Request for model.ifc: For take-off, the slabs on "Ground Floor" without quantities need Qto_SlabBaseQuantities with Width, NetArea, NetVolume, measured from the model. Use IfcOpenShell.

First a look at what the model holds.

```python
import ifcopenshell
import ifcopenshell.util.element
import ifcopenshell.util.unit

model = ifcopenshell.open("model.ifc")
print(model.schema)
for unit_type in ("LENGTHUNIT", "AREAUNIT", "VOLUMEUNIT"):
    print(unit_type, ifcopenshell.util.unit.calculate_unit_scale(model, unit_type))
storey = next(s for s in model.by_type("IfcBuildingStorey") if s.Name == "Ground Floor")
slabs = [e for e in ifcopenshell.util.element.get_decomposition(storey) if e.is_a("IfcSlab")]
for e in sorted(slabs, key=lambda e: e.id()):
    print(e.id(), e.is_a(), e.Name, list(ifcopenshell.util.element.get_psets(e, qtos_only=True)), sep=" | ")
```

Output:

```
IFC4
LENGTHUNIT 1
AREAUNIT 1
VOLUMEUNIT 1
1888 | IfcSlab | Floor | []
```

```python
import ifcopenshell
import ifcopenshell.api.pset
import ifcopenshell.geom
import ifcopenshell.util.element
import ifcopenshell.util.shape
import ifcopenshell.util.unit

model = ifcopenshell.open("model.ifc")
unit_scale = ifcopenshell.util.unit.calculate_unit_scale(model)
area_scale = ifcopenshell.util.unit.calculate_unit_scale(model, "AREAUNIT")
volume_scale = ifcopenshell.util.unit.calculate_unit_scale(model, "VOLUMEUNIT")
settings = ifcopenshell.geom.settings()

storey = next(s for s in model.by_type("IfcBuildingStorey") if s.Name == "Ground Floor")
slabs = [e for e in ifcopenshell.util.element.get_decomposition(storey) if e.is_a("IfcSlab")]

for e in sorted(slabs, key=lambda e: e.id()):
    if ifcopenshell.util.element.get_psets(e, qtos_only=True, should_inherit=False):
        continue
    # Geometry comes back in metres, in the element's own axes.
    shape = ifcopenshell.geom.create_shape(settings, e)
    values = {
        "Width": ifcopenshell.util.shape.get_z(shape.geometry) / unit_scale,
        "NetArea": ifcopenshell.util.shape.get_footprint_area(shape.geometry) / area_scale,
        "NetVolume": ifcopenshell.util.shape.get_volume(shape.geometry) / volume_scale,
    }
    qto = ifcopenshell.api.pset.add_qto(model, product=e, name="Qto_SlabBaseQuantities")
    ifcopenshell.api.pset.edit_qto(model, qto=qto, properties=values)
    print(e.id(), {k: round(v, 3) for k, v in values.items()})

model.write("model_v2.ifc")
```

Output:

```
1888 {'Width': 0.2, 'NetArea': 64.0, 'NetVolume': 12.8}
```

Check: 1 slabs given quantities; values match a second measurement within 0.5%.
